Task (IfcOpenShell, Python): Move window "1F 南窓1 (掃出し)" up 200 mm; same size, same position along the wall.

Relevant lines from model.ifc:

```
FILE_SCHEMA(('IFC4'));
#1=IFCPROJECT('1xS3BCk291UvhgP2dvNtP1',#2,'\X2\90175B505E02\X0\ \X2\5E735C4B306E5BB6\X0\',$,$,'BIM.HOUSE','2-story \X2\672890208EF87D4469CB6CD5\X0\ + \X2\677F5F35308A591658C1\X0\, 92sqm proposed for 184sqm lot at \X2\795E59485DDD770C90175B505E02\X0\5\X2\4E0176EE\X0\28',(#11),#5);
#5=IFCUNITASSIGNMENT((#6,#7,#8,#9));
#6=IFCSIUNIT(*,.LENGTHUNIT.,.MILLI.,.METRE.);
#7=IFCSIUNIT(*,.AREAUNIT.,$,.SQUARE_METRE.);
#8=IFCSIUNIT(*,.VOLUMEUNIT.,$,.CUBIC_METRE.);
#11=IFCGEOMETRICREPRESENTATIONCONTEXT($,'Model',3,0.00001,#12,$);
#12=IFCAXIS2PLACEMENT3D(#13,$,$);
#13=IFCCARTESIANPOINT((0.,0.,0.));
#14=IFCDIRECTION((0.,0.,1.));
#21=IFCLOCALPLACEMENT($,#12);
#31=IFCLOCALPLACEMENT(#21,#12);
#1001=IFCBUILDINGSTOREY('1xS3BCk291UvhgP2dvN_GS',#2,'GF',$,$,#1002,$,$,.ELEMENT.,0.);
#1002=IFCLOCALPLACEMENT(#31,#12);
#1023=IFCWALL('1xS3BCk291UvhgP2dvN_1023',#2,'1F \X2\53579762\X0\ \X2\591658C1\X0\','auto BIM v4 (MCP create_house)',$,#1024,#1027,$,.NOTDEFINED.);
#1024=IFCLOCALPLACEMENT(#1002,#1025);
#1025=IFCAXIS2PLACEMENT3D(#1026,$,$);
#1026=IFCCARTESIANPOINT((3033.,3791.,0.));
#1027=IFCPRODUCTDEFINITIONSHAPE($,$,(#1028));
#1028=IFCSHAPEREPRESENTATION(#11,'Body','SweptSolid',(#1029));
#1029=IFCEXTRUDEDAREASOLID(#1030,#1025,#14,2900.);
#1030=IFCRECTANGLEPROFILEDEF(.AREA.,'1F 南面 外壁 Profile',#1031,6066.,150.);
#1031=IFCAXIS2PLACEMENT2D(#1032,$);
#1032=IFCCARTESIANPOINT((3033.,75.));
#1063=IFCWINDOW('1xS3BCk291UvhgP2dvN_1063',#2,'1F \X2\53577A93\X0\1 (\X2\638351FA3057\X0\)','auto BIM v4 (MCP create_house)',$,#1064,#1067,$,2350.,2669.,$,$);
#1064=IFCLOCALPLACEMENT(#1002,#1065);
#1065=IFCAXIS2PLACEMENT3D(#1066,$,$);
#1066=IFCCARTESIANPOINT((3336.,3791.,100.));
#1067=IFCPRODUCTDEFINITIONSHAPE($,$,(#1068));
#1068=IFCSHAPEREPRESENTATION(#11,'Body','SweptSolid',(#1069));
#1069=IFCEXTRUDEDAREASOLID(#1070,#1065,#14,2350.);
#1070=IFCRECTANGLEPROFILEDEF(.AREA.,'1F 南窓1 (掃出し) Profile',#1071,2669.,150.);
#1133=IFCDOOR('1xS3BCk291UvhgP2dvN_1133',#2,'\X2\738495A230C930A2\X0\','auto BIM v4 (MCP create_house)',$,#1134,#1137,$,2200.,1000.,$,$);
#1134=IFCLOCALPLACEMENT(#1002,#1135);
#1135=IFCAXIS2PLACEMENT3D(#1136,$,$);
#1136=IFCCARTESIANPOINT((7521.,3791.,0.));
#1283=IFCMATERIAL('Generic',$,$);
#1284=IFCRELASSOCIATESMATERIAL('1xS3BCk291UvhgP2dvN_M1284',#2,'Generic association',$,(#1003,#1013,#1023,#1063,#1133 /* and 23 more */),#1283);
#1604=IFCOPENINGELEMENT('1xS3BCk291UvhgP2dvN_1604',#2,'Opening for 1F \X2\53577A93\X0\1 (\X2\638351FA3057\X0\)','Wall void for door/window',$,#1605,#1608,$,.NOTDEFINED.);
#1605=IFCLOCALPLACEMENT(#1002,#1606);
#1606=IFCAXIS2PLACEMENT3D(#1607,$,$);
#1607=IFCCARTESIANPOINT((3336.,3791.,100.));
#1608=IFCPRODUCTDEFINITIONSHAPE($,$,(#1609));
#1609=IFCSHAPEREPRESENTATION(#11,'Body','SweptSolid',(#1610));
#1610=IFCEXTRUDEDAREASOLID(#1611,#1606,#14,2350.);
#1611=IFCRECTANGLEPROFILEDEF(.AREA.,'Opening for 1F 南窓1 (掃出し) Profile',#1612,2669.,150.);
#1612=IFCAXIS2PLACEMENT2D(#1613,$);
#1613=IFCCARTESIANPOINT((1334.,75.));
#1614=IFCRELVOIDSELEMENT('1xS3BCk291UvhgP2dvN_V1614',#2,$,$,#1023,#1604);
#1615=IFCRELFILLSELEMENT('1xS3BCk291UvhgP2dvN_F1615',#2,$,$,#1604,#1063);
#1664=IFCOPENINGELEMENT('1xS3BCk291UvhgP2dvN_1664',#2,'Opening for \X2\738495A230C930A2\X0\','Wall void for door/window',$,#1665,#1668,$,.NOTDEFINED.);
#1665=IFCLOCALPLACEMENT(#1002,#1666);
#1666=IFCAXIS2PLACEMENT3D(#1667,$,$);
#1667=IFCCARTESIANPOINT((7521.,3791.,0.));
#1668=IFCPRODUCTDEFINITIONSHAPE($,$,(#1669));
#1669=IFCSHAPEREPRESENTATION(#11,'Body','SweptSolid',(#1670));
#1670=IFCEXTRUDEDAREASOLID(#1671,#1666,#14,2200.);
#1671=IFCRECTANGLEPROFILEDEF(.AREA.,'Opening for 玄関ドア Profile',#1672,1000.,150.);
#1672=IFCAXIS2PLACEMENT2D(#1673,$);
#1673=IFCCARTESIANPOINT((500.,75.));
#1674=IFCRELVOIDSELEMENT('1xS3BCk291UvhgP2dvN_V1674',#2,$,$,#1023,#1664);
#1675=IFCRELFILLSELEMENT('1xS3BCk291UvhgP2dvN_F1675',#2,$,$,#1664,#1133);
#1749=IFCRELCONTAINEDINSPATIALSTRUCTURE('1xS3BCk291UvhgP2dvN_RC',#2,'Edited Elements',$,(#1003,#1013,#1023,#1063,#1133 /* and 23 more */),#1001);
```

```python
import numpy as np
import ifcopenshell
import ifcopenshell.api.geometry
import ifcopenshell.util.placement
import ifcopenshell.util.unit

model = ifcopenshell.open("model.ifc")
unit_scale = ifcopenshell.util.unit.calculate_unit_scale(model)

window = model.by_guid("1xS3BCk291UvhgP2dvN_1063")
opening = window.FillsVoids[0].RelatingOpeningElement
dz = 0.2 / unit_scale

shift = np.array([0.0, 0.0, dz])
# The window is not placed relative to its opening, so move both.
for product in (opening, window):
    matrix = ifcopenshell.util.placement.get_local_placement(product.ObjectPlacement)
    matrix[:3, 3] += shift
    ifcopenshell.api.geometry.edit_object_placement(model, product=product, matrix=matrix, is_si=False)

print(f"moved by {dz * unit_scale:+.3f} m")

model.write("model_edited.ifc")
```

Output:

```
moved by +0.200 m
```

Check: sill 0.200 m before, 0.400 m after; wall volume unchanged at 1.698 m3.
